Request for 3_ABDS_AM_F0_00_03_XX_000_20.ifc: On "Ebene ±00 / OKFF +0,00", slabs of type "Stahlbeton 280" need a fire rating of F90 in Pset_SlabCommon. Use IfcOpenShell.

First a look at what the model holds.

```python
import ifcopenshell
import ifcopenshell.util.element

model = ifcopenshell.open("3_ABDS_AM_F0_00_03_XX_000_20.ifc")
print(model.schema)
storey = next(s for s in model.by_type("IfcBuildingStorey") if s.Name == "Ebene ±00 / OKFF +0,00")
slabs = [e for e in ifcopenshell.util.element.get_decomposition(storey) if e.is_a("IfcSlab")]
seen = {}
for e in slabs:
    element_type = ifcopenshell.util.element.get_type(e)
    key = (element_type.Name if element_type != e and element_type else None, ifcopenshell.util.element.get_pset(e, "Pset_SlabCommon", "FireRating"))
    seen[key] = seen.get(key, 0) + 1
for (name, value), count in sorted(seen.items(), key=str):
    print(count, "x", name, "|", value)
```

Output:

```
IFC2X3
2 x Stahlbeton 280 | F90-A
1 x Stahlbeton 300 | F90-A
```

```python
import ifcopenshell
import ifcopenshell.api.pset
import ifcopenshell.util.element

model = ifcopenshell.open("3_ABDS_AM_F0_00_03_XX_000_20.ifc")

storey = next(s for s in model.by_type("IfcBuildingStorey") if s.Name == "Ebene ±00 / OKFF +0,00")
slabs = [e for e in ifcopenshell.util.element.get_decomposition(storey) if e.is_a("IfcSlab")]

count = 0
for e in slabs:
    element_type = ifcopenshell.util.element.get_type(e)
    if element_type in (None, e) or element_type.Name != "Stahlbeton 280":
        continue
    # add_pset returns the element's existing set when there is one.
    pset = ifcopenshell.api.pset.add_pset(model, product=e, name="Pset_SlabCommon")
    ifcopenshell.api.pset.edit_pset(model, pset=pset, properties={"FireRating": "F90"})
    count += 1

print(count, "slabs updated")

model.write("3_ABDS_AM_F0_00_03_XX_000_20_v2.ifc")
```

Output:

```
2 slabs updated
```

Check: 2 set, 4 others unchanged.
